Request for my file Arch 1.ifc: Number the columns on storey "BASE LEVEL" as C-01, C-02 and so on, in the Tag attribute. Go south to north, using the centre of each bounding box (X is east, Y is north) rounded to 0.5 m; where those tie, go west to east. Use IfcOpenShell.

First a look at what the model holds.

```python
import ifcopenshell
import ifcopenshell.util.element
import ifcopenshell.util.placement

model = ifcopenshell.open("my file Arch 1.ifc")
print(model.schema)
storey = next(s for s in model.by_type("IfcBuildingStorey") if s.Name == "BASE LEVEL")
columns = [e for e in ifcopenshell.util.element.get_decomposition(storey) if e.is_a("IfcColumn")]
for e in sorted(columns, key=lambda e: e.id()):
    origin = ifcopenshell.util.placement.get_local_placement(e.ObjectPlacement)[:3, 3]
    print(e.id(), e.Tag, e.Name, origin.round(2) + 0.0, sep=" | ")
```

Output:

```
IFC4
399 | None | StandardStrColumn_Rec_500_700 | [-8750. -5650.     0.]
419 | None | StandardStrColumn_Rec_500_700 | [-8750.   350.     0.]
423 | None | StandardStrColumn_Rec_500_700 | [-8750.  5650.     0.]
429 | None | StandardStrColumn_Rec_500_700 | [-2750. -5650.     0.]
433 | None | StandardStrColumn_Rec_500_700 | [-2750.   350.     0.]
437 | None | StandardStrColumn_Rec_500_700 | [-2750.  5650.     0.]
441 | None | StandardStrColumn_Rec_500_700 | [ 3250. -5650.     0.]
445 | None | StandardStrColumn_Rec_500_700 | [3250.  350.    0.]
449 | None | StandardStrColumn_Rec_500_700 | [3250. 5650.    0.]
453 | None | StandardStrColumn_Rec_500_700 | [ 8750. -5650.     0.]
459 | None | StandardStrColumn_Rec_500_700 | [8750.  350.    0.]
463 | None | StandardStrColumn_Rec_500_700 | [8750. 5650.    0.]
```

```python
import ifcopenshell
import ifcopenshell.geom
import ifcopenshell.util.element
import ifcopenshell.util.shape

model = ifcopenshell.open("my file Arch 1.ifc")
settings = ifcopenshell.geom.settings()
settings.set("use-world-coords", True)


def centre(element):
    shape = ifcopenshell.geom.create_shape(settings, element)
    return ifcopenshell.util.shape.get_bbox_centroid(shape.geometry)


storey = next(s for s in model.by_type("IfcBuildingStorey") if s.Name == "BASE LEVEL")
columns = [e for e in ifcopenshell.util.element.get_decomposition(storey) if e.is_a("IfcColumn")]

# Insertion points can sit at a corner or the storey origin, so sort by the geometry (in metres).
centres = {e: centre(e) for e in columns}
columns.sort(key=lambda e: (round(centres[e][1] / 0.5), centres[e][0]))

for i, e in enumerate(columns, start=1):
    number = f"C-{i:02d}"
    e.Tag = number
    print(e.id(), number)

model.write("my file Arch 1_v2.ifc")
```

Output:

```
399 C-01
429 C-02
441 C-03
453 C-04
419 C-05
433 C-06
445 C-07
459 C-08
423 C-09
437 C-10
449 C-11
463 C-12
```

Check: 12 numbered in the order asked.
